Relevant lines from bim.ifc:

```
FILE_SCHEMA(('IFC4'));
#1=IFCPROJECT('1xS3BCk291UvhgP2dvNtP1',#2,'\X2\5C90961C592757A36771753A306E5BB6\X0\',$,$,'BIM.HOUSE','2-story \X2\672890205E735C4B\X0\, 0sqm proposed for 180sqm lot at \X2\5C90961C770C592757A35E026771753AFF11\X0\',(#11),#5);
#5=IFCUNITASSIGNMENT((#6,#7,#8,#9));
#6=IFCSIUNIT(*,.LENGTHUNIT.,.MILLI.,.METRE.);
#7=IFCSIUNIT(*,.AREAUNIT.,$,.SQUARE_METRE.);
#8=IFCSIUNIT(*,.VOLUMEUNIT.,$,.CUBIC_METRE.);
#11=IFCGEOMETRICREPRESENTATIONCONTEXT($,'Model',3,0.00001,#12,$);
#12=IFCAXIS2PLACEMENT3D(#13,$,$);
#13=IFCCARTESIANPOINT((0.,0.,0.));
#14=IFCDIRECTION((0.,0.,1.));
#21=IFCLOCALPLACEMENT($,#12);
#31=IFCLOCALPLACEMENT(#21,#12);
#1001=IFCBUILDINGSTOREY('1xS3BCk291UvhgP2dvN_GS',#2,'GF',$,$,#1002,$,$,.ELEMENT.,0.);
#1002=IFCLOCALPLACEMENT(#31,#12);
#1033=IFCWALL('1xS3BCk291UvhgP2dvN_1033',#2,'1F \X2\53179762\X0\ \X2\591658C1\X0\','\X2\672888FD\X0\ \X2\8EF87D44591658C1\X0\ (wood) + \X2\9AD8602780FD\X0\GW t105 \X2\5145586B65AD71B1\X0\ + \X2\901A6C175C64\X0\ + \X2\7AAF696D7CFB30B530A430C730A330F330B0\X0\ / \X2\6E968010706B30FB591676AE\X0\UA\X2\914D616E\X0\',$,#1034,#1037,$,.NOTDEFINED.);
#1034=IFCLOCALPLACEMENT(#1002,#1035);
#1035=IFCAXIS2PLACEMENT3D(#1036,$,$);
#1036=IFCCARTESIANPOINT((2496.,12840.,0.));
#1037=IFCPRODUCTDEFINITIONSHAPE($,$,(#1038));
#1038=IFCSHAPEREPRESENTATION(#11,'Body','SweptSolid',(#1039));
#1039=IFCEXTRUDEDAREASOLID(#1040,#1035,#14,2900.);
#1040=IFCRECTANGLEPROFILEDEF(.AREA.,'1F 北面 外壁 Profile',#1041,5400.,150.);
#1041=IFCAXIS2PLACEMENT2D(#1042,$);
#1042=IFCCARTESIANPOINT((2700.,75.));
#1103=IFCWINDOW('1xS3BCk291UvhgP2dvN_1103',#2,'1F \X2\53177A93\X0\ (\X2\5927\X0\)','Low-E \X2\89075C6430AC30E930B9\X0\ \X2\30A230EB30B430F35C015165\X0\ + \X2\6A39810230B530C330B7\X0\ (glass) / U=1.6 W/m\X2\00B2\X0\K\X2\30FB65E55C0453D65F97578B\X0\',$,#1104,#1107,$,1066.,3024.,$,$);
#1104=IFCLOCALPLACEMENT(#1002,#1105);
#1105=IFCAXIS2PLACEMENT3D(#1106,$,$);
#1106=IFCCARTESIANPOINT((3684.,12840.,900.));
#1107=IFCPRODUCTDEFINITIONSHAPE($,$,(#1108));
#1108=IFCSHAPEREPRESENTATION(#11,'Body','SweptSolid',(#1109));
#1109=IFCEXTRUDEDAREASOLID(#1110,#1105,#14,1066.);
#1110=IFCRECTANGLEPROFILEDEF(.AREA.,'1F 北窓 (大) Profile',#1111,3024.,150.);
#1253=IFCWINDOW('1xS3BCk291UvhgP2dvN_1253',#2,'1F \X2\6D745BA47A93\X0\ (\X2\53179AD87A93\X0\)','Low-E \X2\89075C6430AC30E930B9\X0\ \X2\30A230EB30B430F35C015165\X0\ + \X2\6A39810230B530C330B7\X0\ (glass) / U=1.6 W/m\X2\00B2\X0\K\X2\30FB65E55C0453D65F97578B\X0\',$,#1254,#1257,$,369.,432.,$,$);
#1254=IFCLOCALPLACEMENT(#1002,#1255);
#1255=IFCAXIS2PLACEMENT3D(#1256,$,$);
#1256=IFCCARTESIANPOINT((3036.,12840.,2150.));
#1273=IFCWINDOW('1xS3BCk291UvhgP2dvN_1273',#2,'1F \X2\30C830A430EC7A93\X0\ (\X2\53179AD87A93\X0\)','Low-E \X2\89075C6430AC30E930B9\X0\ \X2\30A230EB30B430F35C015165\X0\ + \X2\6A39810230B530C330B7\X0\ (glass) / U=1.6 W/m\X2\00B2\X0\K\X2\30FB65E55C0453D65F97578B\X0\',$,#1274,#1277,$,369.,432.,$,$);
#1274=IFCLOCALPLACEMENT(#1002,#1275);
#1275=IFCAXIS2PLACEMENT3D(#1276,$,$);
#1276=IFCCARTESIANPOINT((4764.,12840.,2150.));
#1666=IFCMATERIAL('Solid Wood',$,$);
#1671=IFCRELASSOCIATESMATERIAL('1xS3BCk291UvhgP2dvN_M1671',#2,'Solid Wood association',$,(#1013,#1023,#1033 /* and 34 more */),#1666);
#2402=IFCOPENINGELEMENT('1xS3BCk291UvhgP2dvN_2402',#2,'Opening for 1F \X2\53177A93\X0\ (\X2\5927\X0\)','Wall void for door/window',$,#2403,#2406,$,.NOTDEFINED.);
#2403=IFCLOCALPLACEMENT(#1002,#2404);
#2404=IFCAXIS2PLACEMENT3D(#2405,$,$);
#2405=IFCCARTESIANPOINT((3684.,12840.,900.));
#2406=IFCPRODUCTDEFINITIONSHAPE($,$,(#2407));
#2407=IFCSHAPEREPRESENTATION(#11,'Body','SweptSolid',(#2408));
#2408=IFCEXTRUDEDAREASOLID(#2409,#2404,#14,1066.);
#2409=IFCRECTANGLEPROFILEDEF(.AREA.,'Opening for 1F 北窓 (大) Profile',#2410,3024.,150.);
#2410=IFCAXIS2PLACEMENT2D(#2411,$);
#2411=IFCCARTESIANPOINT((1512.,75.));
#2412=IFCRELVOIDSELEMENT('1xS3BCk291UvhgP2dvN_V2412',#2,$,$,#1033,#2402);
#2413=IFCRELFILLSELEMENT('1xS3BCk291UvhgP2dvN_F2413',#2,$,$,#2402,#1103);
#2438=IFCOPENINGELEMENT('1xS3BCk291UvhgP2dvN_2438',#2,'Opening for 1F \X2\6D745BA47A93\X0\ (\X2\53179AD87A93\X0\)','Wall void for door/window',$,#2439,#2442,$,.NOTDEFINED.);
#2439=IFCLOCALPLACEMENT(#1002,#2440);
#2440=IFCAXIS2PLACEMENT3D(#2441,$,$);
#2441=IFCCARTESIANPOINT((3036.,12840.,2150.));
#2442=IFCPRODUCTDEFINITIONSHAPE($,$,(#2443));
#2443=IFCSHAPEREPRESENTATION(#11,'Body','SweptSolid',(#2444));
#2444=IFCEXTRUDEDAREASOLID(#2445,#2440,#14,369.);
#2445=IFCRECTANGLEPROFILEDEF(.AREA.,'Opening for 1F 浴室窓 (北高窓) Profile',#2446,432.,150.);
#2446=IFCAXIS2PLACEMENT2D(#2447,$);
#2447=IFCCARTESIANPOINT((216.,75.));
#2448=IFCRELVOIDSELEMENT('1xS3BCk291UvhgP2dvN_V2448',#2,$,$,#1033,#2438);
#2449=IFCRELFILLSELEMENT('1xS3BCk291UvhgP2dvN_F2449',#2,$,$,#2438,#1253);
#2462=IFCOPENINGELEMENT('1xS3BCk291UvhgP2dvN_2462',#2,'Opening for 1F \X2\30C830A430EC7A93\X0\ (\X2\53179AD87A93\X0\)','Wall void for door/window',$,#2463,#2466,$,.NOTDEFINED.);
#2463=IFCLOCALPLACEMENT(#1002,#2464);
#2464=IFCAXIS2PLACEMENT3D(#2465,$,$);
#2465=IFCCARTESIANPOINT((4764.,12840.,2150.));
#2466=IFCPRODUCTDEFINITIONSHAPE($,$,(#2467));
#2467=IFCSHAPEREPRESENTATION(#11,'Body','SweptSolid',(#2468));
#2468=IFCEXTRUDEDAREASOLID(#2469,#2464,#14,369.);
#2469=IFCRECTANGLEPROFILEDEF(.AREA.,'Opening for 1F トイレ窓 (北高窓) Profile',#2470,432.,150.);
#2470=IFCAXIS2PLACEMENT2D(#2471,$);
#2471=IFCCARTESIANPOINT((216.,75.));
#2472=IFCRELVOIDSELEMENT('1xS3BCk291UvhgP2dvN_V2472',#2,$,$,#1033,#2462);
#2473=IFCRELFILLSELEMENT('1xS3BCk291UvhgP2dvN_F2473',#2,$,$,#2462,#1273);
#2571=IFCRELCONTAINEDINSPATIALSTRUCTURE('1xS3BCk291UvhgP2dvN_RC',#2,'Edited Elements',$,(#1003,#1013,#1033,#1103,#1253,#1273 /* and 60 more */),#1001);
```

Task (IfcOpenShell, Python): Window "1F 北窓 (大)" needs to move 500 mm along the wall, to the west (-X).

```python
import ifcopenshell
import ifcopenshell.api.geometry
import ifcopenshell.util.placement

model = ifcopenshell.open("bim.ifc")

window = model.by_guid("1xS3BCk291UvhgP2dvN_1103")
opening = window.FillsVoids[0].RelatingOpeningElement
wall = opening.VoidsElements[0].RelatingBuildingElement

wall_matrix = ifcopenshell.util.placement.get_local_placement(wall.ObjectPlacement)
shift = wall_matrix[:3, 0] * -500.0
before = ifcopenshell.util.placement.get_local_placement(window.ObjectPlacement)[:3, 3].copy()

# The window is not placed relative to its opening, so move both.
for product in (opening, window):
    matrix = ifcopenshell.util.placement.get_local_placement(product.ObjectPlacement)
    matrix[:3, 3] += shift
    ifcopenshell.api.geometry.edit_object_placement(model, product=product, matrix=matrix, is_si=False)

after = ifcopenshell.util.placement.get_local_placement(window.ObjectPlacement)[:3, 3]
print("window moved by", (after - before).round(3) + 0.0)

model.write("bim_rev.ifc")
```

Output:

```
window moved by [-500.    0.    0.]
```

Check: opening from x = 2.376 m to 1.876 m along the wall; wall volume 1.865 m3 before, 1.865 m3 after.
